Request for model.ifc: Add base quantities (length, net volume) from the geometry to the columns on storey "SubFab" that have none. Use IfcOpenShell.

First a look at what the model holds.

```python
import ifcopenshell
import ifcopenshell.util.element
import ifcopenshell.util.unit

model = ifcopenshell.open("model.ifc")
print(model.schema)
for unit_type in ("LENGTHUNIT", "AREAUNIT", "VOLUMEUNIT"):
    print(unit_type, ifcopenshell.util.unit.calculate_unit_scale(model, unit_type))
storey = next(s for s in model.by_type("IfcBuildingStorey") if s.Name == "SubFab")
columns = [e for e in ifcopenshell.util.element.get_decomposition(storey) if e.is_a("IfcColumn")]
for e in sorted(columns, key=lambda e: e.id()):
    print(e.id(), e.is_a(), e.Name, list(ifcopenshell.util.element.get_psets(e, qtos_only=True)), sep=" | ")
```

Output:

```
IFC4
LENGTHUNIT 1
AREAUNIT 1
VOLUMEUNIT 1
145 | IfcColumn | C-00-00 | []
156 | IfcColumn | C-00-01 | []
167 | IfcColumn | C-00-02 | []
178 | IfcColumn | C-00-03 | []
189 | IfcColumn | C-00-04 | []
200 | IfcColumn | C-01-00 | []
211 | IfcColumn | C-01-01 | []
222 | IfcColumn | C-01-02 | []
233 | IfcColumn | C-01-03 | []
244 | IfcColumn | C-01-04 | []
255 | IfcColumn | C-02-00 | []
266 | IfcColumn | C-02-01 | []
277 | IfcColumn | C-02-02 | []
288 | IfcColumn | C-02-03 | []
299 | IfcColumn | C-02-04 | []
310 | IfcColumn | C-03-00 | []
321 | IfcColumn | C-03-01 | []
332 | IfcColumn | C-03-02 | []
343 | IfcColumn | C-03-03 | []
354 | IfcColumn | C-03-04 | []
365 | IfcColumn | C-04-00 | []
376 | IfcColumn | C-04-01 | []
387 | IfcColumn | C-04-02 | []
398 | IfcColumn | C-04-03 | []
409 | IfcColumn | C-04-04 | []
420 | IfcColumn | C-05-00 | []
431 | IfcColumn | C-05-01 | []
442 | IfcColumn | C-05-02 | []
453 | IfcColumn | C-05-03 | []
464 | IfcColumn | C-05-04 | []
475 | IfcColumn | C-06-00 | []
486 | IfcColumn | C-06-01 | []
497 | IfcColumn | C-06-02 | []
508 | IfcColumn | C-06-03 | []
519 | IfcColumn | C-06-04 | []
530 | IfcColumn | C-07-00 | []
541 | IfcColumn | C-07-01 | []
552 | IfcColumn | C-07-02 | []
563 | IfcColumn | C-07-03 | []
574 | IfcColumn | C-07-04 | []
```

```python
import ifcopenshell
import ifcopenshell.api.pset
import ifcopenshell.geom
import ifcopenshell.util.element
import ifcopenshell.util.shape
import ifcopenshell.util.unit

model = ifcopenshell.open("model.ifc")
unit_scale = ifcopenshell.util.unit.calculate_unit_scale(model)
volume_scale = ifcopenshell.util.unit.calculate_unit_scale(model, "VOLUMEUNIT")
settings = ifcopenshell.geom.settings()

storey = next(s for s in model.by_type("IfcBuildingStorey") if s.Name == "SubFab")
columns = [e for e in ifcopenshell.util.element.get_decomposition(storey) if e.is_a("IfcColumn")]

for e in sorted(columns, key=lambda e: e.id()):
    if ifcopenshell.util.element.get_psets(e, qtos_only=True, should_inherit=False):
        continue
    # Geometry comes back in metres, in the element's own axes.
    shape = ifcopenshell.geom.create_shape(settings, e)
    values = {
        "Length": ifcopenshell.util.shape.get_z(shape.geometry) / unit_scale,
        "NetVolume": ifcopenshell.util.shape.get_volume(shape.geometry) / volume_scale,
    }
    qto = ifcopenshell.api.pset.add_qto(model, product=e, name="Qto_ColumnBaseQuantities")
    ifcopenshell.api.pset.edit_qto(model, qto=qto, properties=values)
    print(e.id(), {k: round(v, 3) for k, v in values.items()})

model.write("model_rev.ifc")
```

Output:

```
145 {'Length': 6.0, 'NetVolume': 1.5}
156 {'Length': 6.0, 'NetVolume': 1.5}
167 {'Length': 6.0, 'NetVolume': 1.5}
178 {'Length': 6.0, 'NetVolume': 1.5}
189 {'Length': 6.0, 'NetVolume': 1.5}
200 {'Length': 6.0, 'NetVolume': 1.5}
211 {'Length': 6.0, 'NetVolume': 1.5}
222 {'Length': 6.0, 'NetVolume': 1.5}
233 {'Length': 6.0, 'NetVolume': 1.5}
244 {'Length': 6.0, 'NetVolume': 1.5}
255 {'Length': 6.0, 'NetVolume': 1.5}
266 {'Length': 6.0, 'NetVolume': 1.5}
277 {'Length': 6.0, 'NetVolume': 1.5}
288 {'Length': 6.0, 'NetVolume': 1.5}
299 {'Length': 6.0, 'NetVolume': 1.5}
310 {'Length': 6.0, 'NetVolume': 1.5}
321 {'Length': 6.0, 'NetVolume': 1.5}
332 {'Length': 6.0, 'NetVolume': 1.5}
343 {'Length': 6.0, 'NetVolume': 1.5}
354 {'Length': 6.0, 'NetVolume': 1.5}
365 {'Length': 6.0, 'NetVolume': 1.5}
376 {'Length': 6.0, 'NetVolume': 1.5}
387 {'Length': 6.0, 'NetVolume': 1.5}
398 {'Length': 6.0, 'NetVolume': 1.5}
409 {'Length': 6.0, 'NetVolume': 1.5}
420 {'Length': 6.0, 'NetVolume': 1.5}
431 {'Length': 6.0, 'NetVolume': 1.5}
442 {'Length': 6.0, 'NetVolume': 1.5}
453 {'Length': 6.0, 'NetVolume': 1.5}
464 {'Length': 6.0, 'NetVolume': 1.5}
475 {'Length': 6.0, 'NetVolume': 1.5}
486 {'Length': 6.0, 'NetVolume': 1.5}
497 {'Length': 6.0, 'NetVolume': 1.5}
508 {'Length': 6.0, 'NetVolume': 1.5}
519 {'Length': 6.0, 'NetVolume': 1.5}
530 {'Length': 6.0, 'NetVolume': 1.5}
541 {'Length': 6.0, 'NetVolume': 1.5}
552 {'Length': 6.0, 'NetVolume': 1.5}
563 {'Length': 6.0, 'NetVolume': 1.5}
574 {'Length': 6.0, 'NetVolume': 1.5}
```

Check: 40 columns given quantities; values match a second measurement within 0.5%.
